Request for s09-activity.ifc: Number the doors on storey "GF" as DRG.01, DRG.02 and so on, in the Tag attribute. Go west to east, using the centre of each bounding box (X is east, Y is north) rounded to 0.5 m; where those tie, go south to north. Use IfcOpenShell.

First a look at what the model holds.

```python
import ifcopenshell
import ifcopenshell.util.element
import ifcopenshell.util.placement

model = ifcopenshell.open("s09-activity.ifc")
print(model.schema)
storey = next(s for s in model.by_type("IfcBuildingStorey") if s.Name == "GF")
doors = [e for e in ifcopenshell.util.element.get_decomposition(storey) if e.is_a("IfcDoor")]
for e in sorted(doors, key=lambda e: e.id()):
    origin = ifcopenshell.util.placement.get_local_placement(e.ObjectPlacement)[:3, 3]
    print(e.id(), e.Tag, e.Name, origin.round(2) + 0.0, sep=" | ")
```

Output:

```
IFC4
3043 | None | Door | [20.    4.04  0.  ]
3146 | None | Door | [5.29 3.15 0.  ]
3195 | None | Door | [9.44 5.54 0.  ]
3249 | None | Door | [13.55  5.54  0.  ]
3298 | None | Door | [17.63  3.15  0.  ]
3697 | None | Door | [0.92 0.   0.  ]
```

```python
import ifcopenshell
import ifcopenshell.geom
import ifcopenshell.util.element
import ifcopenshell.util.shape

model = ifcopenshell.open("s09-activity.ifc")
settings = ifcopenshell.geom.settings()
settings.set("use-world-coords", True)


def centre(element):
    shape = ifcopenshell.geom.create_shape(settings, element)
    return ifcopenshell.util.shape.get_bbox_centroid(shape.geometry)


storey = next(s for s in model.by_type("IfcBuildingStorey") if s.Name == "GF")
doors = [e for e in ifcopenshell.util.element.get_decomposition(storey) if e.is_a("IfcDoor")]

# Insertion points can sit at a corner or the storey origin, so sort by the geometry (in metres).
centres = {e: centre(e) for e in doors}
doors.sort(key=lambda e: (round(centres[e][0] / 0.5), centres[e][1]))

for i, e in enumerate(doors, start=1):
    number = f"DRG.{i:02d}"
    e.Tag = number
    print(e.id(), number)

model.write("s09-activity_edited.ifc")
```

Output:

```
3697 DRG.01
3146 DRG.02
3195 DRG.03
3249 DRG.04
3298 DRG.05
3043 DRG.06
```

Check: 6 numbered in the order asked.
